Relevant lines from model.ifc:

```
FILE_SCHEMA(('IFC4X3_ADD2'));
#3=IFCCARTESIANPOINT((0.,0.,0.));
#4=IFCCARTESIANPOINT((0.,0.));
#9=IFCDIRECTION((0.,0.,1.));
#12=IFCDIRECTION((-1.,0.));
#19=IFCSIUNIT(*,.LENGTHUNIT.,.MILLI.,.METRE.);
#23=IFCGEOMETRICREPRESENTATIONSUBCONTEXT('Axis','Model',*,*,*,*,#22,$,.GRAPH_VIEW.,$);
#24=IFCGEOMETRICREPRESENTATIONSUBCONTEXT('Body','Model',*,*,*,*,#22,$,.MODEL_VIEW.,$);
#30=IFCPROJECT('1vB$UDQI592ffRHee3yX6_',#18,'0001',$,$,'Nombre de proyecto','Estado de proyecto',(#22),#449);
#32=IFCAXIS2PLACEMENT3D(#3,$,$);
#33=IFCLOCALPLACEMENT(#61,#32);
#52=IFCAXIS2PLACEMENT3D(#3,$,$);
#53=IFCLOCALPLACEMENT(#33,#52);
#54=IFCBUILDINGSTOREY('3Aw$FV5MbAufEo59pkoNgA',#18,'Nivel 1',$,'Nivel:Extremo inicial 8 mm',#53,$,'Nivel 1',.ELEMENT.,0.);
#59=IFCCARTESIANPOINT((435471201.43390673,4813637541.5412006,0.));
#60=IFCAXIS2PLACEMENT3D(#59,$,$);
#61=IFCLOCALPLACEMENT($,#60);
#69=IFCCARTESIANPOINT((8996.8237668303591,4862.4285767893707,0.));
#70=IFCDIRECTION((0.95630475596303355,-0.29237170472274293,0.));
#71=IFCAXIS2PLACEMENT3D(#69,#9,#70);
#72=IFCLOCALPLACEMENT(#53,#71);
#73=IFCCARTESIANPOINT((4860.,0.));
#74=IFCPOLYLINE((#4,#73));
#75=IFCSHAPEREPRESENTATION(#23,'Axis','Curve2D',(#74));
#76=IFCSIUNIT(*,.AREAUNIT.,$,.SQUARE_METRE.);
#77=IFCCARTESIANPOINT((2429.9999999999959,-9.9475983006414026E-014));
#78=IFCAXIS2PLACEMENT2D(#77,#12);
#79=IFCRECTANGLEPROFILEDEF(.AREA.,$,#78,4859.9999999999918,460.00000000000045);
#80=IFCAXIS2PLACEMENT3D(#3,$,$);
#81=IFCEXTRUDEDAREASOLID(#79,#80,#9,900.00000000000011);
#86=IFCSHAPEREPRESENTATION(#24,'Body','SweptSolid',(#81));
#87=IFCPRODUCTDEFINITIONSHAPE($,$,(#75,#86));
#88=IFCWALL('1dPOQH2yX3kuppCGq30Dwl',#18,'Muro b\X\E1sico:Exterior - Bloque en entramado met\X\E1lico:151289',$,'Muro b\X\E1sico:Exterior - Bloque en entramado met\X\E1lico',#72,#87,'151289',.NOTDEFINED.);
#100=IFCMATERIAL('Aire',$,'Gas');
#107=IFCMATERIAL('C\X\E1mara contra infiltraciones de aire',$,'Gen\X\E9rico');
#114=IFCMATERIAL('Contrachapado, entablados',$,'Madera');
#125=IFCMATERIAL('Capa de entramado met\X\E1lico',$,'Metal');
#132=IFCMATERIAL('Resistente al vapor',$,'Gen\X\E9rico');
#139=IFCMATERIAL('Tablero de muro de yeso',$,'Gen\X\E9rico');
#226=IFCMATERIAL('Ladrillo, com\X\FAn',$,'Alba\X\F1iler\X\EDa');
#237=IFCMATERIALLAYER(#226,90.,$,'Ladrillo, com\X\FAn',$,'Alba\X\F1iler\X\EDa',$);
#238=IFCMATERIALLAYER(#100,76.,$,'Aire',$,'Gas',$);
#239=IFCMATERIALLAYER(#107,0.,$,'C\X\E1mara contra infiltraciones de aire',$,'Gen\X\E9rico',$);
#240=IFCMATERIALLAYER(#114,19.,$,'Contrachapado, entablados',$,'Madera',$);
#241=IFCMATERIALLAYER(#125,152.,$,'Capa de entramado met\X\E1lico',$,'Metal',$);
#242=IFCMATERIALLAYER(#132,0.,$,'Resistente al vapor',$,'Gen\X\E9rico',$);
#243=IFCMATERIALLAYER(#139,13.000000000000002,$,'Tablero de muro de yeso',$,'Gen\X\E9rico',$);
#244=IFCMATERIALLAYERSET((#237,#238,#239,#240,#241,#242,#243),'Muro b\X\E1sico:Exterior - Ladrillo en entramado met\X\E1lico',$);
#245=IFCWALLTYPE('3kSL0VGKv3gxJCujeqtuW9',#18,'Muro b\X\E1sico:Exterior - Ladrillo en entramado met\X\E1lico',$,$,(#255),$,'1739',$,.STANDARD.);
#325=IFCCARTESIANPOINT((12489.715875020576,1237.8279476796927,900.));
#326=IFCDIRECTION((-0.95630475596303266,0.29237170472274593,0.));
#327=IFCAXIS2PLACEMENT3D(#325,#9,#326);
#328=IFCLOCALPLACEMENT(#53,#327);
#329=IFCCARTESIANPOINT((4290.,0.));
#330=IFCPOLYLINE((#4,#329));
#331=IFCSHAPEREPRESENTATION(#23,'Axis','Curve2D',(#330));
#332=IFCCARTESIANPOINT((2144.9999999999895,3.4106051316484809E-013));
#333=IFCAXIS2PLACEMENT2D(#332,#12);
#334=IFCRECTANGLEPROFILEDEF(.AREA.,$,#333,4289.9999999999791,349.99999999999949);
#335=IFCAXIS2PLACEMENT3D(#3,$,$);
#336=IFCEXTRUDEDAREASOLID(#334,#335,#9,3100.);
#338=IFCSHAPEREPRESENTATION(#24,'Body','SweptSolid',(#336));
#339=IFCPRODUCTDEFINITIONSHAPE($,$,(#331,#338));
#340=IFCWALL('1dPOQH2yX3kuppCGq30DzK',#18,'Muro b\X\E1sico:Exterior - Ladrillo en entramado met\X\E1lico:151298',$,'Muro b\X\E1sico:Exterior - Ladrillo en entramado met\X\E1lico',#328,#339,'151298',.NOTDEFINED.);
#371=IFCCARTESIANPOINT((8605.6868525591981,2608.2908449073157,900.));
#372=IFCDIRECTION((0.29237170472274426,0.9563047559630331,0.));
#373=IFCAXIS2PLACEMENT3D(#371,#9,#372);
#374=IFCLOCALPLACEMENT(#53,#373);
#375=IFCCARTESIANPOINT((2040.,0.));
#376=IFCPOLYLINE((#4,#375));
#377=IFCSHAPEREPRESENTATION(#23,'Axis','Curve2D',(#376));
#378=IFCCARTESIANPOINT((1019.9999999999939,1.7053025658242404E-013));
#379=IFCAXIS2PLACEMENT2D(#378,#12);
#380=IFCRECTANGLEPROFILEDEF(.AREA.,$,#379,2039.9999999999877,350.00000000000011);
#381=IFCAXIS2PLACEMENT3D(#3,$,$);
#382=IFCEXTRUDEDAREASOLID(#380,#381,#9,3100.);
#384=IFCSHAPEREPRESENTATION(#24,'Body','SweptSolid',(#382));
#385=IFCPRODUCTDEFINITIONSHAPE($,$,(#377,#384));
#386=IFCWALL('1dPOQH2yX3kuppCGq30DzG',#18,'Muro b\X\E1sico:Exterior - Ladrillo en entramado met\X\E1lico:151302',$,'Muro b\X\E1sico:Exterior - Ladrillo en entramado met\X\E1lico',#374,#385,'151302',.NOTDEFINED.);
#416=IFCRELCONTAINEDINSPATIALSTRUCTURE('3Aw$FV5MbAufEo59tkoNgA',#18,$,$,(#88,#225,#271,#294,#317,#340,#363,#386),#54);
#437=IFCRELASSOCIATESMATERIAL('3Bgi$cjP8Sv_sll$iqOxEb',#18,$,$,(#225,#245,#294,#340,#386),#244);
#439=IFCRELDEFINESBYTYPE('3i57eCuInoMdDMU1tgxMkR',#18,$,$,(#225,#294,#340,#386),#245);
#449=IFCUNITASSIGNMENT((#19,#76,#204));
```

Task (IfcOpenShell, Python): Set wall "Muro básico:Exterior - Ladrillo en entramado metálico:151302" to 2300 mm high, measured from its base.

```python
import ifcopenshell
import ifcopenshell.geom
import ifcopenshell.util.representation
import ifcopenshell.util.shape

model = ifcopenshell.open("model.ifc")
settings = ifcopenshell.geom.settings()


def volume(element):
    """Net volume in cubic metres, openings subtracted."""
    shape = ifcopenshell.geom.create_shape(settings, element)
    return ifcopenshell.util.shape.get_volume(shape.geometry)


wall = model.by_id(386)
before = volume(wall)

body = ifcopenshell.util.representation.get_representation(wall, "Model", "Body")
solid = body.Items[0]
old_height = solid.Depth
solid.Depth = 2300.0
after = volume(wall)

print(f"height {old_height:g} -> {solid.Depth:g}, volume {before:.3f} -> {after:.3f} m3")

model.write("model-out.ifc")
```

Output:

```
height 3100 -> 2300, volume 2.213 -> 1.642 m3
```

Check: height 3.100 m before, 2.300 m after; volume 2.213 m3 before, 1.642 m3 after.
